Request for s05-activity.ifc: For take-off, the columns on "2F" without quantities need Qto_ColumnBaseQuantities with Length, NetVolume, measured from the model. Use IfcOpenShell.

First a look at what the model holds.

```python
import ifcopenshell
import ifcopenshell.util.element
import ifcopenshell.util.unit

model = ifcopenshell.open("s05-activity.ifc")
print(model.schema)
for unit_type in ("LENGTHUNIT", "AREAUNIT", "VOLUMEUNIT"):
    print(unit_type, ifcopenshell.util.unit.calculate_unit_scale(model, unit_type))
storey = next(s for s in model.by_type("IfcBuildingStorey") if s.Name == "2F")
columns = [e for e in ifcopenshell.util.element.get_decomposition(storey) if e.is_a("IfcColumn")]
for e in sorted(columns, key=lambda e: e.id()):
    print(e.id(), e.is_a(), e.Name, list(ifcopenshell.util.element.get_psets(e, qtos_only=True)), sep=" | ")
```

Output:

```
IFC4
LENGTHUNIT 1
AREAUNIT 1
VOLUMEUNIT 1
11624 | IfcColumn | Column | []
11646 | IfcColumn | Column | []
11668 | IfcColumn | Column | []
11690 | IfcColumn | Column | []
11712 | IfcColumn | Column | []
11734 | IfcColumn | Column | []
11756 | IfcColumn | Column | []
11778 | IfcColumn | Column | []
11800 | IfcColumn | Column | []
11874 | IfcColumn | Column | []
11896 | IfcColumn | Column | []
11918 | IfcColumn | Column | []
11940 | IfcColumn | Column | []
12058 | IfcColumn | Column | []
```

```python
import ifcopenshell
import ifcopenshell.api.pset
import ifcopenshell.geom
import ifcopenshell.util.element
import ifcopenshell.util.shape
import ifcopenshell.util.unit

model = ifcopenshell.open("s05-activity.ifc")
unit_scale = ifcopenshell.util.unit.calculate_unit_scale(model)
volume_scale = ifcopenshell.util.unit.calculate_unit_scale(model, "VOLUMEUNIT")
settings = ifcopenshell.geom.settings()

storey = next(s for s in model.by_type("IfcBuildingStorey") if s.Name == "2F")
columns = [e for e in ifcopenshell.util.element.get_decomposition(storey) if e.is_a("IfcColumn")]

for e in sorted(columns, key=lambda e: e.id()):
    if ifcopenshell.util.element.get_psets(e, qtos_only=True, should_inherit=False):
        continue
    # Geometry comes back in metres, in the element's own axes.
    shape = ifcopenshell.geom.create_shape(settings, e)
    values = {
        "Length": ifcopenshell.util.shape.get_z(shape.geometry) / unit_scale,
        "NetVolume": ifcopenshell.util.shape.get_volume(shape.geometry) / volume_scale,
    }
    qto = ifcopenshell.api.pset.add_qto(model, product=e, name="Qto_ColumnBaseQuantities")
    ifcopenshell.api.pset.edit_qto(model, qto=qto, properties=values)
    print(e.id(), {k: round(v, 3) for k, v in values.items()})

model.write("s05-activity_updated.ifc")
```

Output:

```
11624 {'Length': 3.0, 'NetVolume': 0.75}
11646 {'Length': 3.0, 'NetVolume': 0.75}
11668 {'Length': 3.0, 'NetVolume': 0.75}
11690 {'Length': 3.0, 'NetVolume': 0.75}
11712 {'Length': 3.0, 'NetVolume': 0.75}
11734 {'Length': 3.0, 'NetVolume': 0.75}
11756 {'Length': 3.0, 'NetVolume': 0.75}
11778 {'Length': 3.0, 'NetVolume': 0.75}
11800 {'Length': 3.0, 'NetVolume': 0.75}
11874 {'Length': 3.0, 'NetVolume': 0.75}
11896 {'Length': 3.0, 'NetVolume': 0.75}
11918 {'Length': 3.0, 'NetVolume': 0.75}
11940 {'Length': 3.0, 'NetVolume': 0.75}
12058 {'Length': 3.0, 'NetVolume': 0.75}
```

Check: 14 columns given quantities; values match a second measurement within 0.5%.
